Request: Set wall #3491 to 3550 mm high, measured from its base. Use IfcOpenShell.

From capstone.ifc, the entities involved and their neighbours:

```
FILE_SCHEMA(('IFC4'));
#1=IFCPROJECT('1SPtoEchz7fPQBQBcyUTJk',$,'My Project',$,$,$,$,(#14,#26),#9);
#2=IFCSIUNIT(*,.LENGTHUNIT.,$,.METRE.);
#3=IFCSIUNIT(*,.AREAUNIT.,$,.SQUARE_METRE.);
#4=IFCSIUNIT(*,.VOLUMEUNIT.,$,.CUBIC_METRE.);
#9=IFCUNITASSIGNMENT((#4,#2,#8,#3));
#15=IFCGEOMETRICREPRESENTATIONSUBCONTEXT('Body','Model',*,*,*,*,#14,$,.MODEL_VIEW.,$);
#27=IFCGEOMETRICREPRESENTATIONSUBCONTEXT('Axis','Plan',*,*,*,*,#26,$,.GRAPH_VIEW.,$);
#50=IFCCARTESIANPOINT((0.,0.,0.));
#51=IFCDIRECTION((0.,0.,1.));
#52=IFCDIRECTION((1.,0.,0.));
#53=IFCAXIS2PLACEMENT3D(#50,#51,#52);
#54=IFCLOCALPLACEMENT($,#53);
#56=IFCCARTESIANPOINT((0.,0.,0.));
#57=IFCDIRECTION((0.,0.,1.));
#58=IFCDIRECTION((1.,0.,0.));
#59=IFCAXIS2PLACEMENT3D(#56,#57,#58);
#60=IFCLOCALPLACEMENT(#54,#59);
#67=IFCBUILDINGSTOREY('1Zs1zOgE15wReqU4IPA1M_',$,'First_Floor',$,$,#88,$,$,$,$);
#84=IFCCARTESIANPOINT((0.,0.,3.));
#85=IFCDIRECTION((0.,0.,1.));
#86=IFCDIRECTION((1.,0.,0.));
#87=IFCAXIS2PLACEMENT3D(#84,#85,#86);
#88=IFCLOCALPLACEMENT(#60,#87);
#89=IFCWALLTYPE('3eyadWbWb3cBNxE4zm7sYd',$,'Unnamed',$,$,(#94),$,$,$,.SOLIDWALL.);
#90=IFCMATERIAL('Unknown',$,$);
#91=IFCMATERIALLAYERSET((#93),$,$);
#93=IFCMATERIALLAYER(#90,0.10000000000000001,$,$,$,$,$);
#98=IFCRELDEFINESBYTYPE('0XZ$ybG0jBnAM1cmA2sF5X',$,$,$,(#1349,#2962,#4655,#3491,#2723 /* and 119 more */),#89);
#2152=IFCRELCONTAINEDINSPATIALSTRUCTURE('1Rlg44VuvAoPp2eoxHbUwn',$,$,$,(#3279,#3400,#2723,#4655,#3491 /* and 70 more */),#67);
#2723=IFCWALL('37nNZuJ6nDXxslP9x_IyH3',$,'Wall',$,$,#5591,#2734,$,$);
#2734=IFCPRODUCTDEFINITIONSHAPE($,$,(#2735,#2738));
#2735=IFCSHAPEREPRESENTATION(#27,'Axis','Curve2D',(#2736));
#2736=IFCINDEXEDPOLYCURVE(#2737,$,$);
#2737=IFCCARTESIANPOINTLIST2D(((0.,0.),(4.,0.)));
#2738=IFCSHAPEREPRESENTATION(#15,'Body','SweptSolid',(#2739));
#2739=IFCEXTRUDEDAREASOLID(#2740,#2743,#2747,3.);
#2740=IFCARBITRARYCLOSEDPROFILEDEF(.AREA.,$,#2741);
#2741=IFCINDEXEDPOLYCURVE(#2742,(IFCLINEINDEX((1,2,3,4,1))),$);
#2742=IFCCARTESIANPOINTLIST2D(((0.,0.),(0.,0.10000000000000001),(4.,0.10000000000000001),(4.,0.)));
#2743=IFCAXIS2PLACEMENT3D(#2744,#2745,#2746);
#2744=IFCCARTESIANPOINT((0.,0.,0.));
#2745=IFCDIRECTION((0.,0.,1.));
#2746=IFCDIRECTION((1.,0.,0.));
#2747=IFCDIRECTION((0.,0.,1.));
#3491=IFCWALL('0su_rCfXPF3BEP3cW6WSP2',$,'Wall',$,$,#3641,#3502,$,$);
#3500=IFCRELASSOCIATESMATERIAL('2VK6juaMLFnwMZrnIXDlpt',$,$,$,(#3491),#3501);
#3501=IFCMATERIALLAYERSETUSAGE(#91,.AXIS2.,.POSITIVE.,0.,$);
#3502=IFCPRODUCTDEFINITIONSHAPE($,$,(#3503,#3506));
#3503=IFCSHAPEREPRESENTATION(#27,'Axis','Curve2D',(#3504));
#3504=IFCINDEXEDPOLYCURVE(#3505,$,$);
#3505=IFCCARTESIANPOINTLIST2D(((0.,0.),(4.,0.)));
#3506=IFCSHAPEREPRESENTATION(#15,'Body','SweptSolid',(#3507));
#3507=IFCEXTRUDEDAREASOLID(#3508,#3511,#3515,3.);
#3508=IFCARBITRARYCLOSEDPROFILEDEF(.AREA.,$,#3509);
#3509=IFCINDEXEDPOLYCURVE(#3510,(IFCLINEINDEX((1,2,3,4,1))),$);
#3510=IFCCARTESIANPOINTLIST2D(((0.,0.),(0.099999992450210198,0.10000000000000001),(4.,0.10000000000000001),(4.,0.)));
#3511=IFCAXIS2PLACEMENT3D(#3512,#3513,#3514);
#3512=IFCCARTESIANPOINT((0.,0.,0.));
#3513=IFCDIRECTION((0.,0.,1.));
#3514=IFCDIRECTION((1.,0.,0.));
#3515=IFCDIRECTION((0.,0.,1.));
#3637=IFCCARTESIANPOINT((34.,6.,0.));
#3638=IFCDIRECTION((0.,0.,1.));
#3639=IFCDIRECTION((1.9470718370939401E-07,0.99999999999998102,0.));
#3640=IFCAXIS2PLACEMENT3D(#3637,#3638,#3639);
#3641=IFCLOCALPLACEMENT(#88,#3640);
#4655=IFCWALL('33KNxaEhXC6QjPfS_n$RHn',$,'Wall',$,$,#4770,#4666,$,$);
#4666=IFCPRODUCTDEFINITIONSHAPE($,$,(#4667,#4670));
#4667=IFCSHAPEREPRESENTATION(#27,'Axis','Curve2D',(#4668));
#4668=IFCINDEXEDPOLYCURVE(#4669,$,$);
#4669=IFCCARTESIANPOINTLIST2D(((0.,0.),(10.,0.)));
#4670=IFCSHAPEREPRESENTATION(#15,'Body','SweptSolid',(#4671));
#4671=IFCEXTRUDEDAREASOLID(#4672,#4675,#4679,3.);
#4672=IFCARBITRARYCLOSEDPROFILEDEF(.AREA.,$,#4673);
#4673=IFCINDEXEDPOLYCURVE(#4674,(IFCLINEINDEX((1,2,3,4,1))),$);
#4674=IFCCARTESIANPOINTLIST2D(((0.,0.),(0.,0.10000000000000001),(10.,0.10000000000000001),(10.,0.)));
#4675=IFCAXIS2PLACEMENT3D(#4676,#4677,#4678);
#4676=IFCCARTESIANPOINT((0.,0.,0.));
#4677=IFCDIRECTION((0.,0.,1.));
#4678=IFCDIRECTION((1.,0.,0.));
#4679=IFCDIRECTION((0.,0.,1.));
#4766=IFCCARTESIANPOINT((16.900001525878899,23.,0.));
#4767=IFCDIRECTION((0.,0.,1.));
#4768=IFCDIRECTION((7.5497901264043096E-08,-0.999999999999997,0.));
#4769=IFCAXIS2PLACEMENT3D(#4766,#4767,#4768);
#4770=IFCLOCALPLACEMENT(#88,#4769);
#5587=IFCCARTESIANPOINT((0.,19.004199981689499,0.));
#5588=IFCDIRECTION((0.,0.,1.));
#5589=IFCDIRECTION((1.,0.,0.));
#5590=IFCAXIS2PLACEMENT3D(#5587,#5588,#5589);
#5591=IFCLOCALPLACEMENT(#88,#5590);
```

```python
import ifcopenshell
import ifcopenshell.geom
import ifcopenshell.util.representation
import ifcopenshell.util.shape

model = ifcopenshell.open("capstone.ifc")
settings = ifcopenshell.geom.settings()


def volume(element):
    """Net volume in cubic metres, openings subtracted."""
    shape = ifcopenshell.geom.create_shape(settings, element)
    return ifcopenshell.util.shape.get_volume(shape.geometry)


wall = model.by_guid("0su_rCfXPF3BEP3cW6WSP2")
before = volume(wall)

body = ifcopenshell.util.representation.get_representation(wall, "Model", "Body")
solid = body.Items[0]
old_height = solid.Depth
solid.Depth = 3.55
after = volume(wall)

print(f"height {old_height:g} -> {solid.Depth:g}, volume {before:.3f} -> {after:.3f} m3")

model.write("capstone-out.ifc")
```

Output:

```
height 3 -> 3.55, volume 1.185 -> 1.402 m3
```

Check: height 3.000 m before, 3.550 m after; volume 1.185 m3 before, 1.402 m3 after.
